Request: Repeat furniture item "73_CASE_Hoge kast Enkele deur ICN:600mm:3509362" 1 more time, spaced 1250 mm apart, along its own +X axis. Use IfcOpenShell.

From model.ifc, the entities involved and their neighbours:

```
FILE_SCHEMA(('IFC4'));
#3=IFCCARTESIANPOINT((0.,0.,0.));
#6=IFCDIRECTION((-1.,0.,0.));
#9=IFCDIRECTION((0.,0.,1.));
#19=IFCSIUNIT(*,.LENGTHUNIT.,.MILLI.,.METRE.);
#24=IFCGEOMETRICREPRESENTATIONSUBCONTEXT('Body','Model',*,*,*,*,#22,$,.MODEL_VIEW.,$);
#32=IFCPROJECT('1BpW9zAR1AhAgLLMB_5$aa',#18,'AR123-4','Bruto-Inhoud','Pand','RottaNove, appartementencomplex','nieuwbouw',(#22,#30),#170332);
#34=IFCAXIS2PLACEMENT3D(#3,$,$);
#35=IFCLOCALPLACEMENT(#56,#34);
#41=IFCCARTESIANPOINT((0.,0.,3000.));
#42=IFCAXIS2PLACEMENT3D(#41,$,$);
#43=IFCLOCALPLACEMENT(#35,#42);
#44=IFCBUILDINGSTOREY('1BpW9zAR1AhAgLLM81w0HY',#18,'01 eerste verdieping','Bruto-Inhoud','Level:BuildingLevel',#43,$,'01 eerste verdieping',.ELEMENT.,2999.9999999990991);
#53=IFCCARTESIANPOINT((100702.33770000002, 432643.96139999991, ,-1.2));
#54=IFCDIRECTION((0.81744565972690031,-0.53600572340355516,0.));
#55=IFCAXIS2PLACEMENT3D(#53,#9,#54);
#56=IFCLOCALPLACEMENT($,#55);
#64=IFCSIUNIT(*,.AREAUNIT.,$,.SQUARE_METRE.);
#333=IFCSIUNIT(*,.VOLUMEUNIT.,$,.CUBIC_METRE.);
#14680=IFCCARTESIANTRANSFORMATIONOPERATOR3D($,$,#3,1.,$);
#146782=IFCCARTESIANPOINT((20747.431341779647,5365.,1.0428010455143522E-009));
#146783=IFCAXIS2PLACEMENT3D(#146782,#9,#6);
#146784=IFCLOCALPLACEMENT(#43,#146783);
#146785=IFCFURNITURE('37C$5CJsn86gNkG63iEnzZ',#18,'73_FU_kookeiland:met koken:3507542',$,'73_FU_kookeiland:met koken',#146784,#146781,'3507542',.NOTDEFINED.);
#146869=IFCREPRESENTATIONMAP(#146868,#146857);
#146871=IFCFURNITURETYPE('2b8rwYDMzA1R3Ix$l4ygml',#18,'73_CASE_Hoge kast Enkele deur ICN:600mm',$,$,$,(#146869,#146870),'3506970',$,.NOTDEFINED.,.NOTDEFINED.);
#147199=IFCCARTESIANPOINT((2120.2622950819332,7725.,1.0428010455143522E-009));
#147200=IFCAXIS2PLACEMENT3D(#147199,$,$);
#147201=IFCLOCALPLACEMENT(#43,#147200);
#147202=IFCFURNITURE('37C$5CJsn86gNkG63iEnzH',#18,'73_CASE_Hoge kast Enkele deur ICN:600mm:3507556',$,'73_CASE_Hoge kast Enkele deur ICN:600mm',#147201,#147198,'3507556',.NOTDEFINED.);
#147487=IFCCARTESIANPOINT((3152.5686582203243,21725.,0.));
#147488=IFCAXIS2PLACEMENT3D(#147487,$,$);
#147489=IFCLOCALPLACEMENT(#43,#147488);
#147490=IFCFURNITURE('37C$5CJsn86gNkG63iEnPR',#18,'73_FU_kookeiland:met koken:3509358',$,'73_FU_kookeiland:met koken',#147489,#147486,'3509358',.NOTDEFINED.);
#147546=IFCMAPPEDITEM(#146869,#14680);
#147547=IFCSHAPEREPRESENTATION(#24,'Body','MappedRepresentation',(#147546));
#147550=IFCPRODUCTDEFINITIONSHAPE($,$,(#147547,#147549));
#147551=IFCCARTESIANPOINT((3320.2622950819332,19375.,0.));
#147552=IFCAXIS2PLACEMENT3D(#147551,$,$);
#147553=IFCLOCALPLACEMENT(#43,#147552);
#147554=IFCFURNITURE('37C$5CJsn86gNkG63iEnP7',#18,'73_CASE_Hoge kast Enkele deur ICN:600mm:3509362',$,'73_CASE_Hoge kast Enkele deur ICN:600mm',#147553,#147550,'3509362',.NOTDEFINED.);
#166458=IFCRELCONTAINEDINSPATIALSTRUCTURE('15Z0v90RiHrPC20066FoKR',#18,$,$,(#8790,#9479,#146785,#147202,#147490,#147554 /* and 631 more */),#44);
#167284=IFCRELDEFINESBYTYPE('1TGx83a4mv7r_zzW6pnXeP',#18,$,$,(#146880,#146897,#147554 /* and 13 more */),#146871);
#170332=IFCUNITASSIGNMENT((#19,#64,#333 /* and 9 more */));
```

```python
import ifcopenshell
import ifcopenshell.api.geometry
import ifcopenshell.api.root
import ifcopenshell.util.element
import ifcopenshell.util.placement

model = ifcopenshell.open("model.ifc")


def reuse_history(source, copy):
    """copy_class also copies each property set's owner history, people and application; keep the originals."""
    for rel in copy.IsDefinedBy:
        if rel.is_a("IfcRelDefinesByProperties") and (history := rel.RelatingPropertyDefinition.OwnerHistory):
            rel.RelatingPropertyDefinition.OwnerHistory = source.OwnerHistory
            ifcopenshell.util.element.remove_deep2(model, history)


source = model.by_guid("37C$5CJsn86gNkG63iEnP7")
base = ifcopenshell.util.placement.get_local_placement(source.ObjectPlacement)
step = base[:3, 0] * 1250.0

for i in range(1, 2):
    copy = ifcopenshell.api.root.copy_class(model, product=source)
    copy.Representation = ifcopenshell.util.element.copy_deep(
        model, source.Representation, exclude=["IfcGeometricRepresentationContext", "IfcRepresentationMap"]
    )
    copy.Name = "73_CASE_Hoge kast Enkele deur ICN:600mm"
    copy.Tag = None
    reuse_history(source, copy)
    matrix = base.copy()
    matrix[:3, 3] += i * step
    print("added at", matrix[:3, 3].round(3) + 0.0)
    ifcopenshell.api.geometry.edit_object_placement(model, product=copy, matrix=matrix, is_si=False)

model.write("model-out.ifc")
```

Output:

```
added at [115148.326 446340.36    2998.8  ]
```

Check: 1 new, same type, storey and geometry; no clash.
